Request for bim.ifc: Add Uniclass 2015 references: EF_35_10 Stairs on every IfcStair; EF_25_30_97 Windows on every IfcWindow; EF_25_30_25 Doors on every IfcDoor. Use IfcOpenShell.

First a look at what the model holds.

```python
import ifcopenshell

model = ifcopenshell.open("bim.ifc")
print(model.schema)
print("classifications:", [c.Name for c in model.by_type("IfcClassification")])
for ifc_class in ("IfcDoor", "IfcRoof", "IfcStair", "IfcWall", "IfcWindow"):
    print(ifc_class, len(model.by_type(ifc_class)))
```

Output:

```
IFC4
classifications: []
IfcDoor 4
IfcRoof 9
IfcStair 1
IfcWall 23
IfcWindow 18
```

```python
import ifcopenshell
import ifcopenshell.api.classification

model = ifcopenshell.open("bim.ifc")

system = ifcopenshell.api.classification.add_classification(model, classification="Uniclass 2015")

codes = {
    "IfcStair": ("EF_35_10", "Stairs"),
    "IfcWindow": ("EF_25_30_97", "Windows"),
    "IfcDoor": ("EF_25_30_25", "Doors"),
}
for ifc_class, (code, name) in codes.items():
    products = model.by_type(ifc_class)
    ifcopenshell.api.classification.add_reference(
        model, products=products, classification=system, identification=code, name=name
    )
    print(code, len(products))

model.write("bim-out.ifc")
```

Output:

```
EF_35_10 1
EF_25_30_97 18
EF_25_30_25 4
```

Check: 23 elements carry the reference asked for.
